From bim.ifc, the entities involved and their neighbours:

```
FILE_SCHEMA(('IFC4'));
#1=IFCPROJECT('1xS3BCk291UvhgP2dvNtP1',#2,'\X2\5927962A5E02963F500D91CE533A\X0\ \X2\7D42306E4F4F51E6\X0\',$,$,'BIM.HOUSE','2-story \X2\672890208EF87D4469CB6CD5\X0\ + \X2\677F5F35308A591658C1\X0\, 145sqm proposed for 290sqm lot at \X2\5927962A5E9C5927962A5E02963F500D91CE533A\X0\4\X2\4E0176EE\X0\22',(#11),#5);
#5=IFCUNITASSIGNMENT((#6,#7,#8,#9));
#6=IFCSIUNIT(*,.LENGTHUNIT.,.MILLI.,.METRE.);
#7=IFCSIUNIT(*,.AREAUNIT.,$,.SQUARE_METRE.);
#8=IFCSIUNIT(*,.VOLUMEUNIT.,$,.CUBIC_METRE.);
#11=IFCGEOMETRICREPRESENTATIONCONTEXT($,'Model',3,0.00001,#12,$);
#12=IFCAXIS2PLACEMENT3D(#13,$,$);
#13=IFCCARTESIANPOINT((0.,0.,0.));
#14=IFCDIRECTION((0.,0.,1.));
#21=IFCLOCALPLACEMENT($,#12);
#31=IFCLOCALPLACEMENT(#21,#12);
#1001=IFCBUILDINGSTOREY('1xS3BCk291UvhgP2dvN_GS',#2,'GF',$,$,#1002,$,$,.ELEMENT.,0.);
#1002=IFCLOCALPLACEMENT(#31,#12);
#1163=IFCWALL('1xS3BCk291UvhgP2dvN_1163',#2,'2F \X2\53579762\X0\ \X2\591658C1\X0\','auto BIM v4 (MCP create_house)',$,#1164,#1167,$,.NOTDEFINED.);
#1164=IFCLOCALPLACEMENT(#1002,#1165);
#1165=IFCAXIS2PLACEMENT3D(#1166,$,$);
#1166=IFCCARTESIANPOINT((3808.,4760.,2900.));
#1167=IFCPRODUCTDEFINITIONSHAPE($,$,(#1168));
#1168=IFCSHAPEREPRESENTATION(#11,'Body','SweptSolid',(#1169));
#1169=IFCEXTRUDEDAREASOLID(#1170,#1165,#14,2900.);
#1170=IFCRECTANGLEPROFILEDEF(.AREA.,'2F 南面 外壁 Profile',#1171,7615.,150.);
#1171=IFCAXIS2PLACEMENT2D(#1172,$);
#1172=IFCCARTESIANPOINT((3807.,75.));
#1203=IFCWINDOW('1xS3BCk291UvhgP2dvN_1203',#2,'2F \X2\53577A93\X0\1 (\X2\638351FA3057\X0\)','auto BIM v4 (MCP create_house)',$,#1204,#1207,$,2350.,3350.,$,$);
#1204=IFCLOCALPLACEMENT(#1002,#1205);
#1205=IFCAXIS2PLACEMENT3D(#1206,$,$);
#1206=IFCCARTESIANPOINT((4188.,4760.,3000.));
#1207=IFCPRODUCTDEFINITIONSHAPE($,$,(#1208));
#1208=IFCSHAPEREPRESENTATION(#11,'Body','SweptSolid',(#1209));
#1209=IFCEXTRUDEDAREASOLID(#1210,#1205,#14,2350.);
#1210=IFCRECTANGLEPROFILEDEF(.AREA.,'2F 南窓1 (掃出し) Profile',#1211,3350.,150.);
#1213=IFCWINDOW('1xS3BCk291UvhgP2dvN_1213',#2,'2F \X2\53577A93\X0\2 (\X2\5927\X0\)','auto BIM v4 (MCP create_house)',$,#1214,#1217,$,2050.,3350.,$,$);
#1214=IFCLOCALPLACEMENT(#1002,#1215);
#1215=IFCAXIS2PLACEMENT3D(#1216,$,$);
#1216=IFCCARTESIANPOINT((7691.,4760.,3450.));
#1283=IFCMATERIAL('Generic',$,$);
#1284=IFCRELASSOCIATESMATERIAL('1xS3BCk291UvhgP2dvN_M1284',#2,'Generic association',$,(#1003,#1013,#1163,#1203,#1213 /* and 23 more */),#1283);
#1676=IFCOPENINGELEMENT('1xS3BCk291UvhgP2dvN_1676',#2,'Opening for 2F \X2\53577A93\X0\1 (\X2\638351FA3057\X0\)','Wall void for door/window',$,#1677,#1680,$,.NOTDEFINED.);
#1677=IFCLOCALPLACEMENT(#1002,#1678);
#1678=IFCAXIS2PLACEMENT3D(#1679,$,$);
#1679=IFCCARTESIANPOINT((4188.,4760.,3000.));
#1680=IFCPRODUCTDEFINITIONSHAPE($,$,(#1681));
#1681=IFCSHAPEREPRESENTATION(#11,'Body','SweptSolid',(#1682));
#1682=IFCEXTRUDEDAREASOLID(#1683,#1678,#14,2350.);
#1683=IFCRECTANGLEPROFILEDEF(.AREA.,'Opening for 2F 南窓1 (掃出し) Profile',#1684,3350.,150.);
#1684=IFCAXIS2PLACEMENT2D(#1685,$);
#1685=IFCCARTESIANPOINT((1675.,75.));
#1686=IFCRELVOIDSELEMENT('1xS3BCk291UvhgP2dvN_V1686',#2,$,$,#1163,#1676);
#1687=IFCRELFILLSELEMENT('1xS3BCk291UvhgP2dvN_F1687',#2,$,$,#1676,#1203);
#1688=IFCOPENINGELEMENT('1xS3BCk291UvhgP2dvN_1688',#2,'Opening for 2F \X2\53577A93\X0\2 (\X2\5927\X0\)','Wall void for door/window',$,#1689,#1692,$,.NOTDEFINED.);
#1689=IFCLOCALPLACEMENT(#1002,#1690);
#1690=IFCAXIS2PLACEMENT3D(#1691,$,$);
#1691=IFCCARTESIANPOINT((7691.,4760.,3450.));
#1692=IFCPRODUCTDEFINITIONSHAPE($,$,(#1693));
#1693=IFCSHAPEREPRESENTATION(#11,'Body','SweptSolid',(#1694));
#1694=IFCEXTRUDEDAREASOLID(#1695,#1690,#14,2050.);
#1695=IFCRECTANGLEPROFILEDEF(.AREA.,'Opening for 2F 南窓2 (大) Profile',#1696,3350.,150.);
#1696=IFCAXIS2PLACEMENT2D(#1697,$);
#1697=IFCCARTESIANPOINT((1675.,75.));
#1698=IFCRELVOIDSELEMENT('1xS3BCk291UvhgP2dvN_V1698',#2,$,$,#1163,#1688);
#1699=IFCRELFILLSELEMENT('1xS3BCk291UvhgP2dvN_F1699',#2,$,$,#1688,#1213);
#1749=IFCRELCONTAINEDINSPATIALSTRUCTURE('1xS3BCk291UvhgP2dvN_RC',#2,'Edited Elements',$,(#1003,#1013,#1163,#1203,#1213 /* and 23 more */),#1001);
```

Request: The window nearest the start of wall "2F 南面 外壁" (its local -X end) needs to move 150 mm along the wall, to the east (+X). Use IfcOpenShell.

```python
import ifcopenshell
import ifcopenshell.api.geometry
import ifcopenshell.util.placement
import ifcopenshell.util.unit

model = ifcopenshell.open("bim.ifc")
unit_scale = ifcopenshell.util.unit.calculate_unit_scale(model)

window = model.by_id(1203)
opening = window.FillsVoids[0].RelatingOpeningElement
wall = opening.VoidsElements[0].RelatingBuildingElement

wall_matrix = ifcopenshell.util.placement.get_local_placement(wall.ObjectPlacement)
shift = wall_matrix[:3, 0] * 0.15 / unit_scale
before = ifcopenshell.util.placement.get_local_placement(window.ObjectPlacement)[:3, 3].copy()

# The window is not placed relative to its opening, so move both.
for product in (opening, window):
    matrix = ifcopenshell.util.placement.get_local_placement(product.ObjectPlacement)
    matrix[:3, 3] += shift
    ifcopenshell.api.geometry.edit_object_placement(model, product=product, matrix=matrix, is_si=False)

after = ifcopenshell.util.placement.get_local_placement(window.ObjectPlacement)[:3, 3]
print("window moved by", (after - before).round(3) + 0.0)

model.write("bim_v2.ifc")
```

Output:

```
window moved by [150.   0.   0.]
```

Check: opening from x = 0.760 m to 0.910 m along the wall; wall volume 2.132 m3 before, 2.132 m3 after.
